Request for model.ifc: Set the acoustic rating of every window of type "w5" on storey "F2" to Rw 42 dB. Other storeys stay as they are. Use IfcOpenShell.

First a look at what the model holds.

```python
import ifcopenshell
import ifcopenshell.util.element

model = ifcopenshell.open("model.ifc")
print(model.schema)
storey = next(s for s in model.by_type("IfcBuildingStorey") if s.Name == "F2")
windows = [e for e in ifcopenshell.util.element.get_decomposition(storey) if e.is_a("IfcWindow")]
seen = {}
for e in windows:
    element_type = ifcopenshell.util.element.get_type(e)
    key = (element_type.Name if element_type != e and element_type else None, ifcopenshell.util.element.get_pset(e, "Pset_WindowCommon", "AcousticRating"))
    seen[key] = seen.get(key, 0) + 1
for (name, value), count in sorted(seen.items(), key=str):
    print(count, "x", name, "|", value)
```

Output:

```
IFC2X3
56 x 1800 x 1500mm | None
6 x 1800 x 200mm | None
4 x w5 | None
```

```python
import ifcopenshell
import ifcopenshell.api.pset
import ifcopenshell.util.element

model = ifcopenshell.open("model.ifc")

storey = next(s for s in model.by_type("IfcBuildingStorey") if s.Name == "F2")
windows = [e for e in ifcopenshell.util.element.get_decomposition(storey) if e.is_a("IfcWindow")]

count = 0
for e in windows:
    element_type = ifcopenshell.util.element.get_type(e)
    if element_type in (None, e) or element_type.Name != "w5":
        continue
    # add_pset returns the element's existing set when there is one.
    pset = ifcopenshell.api.pset.add_pset(model, product=e, name="Pset_WindowCommon")
    ifcopenshell.api.pset.edit_pset(model, pset=pset, properties={"AcousticRating": "Rw 42 dB"})
    count += 1

print(count, "windows updated")

model.write("model_edited.ifc")
```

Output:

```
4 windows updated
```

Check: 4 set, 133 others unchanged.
